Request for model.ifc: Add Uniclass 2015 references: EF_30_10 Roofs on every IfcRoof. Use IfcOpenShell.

First a look at what the model holds.

```python
import ifcopenshell

model = ifcopenshell.open("model.ifc")
print(model.schema)
print("classifications:", [c.Name for c in model.by_type("IfcClassification")])
for ifc_class in ("IfcDoor", "IfcRoof", "IfcStair", "IfcWall", "IfcWindow"):
    print(ifc_class, len(model.by_type(ifc_class)))
```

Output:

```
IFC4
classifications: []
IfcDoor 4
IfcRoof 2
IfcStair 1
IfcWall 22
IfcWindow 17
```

```python
import ifcopenshell
import ifcopenshell.api.classification

model = ifcopenshell.open("model.ifc")

system = ifcopenshell.api.classification.add_classification(model, classification="Uniclass 2015")

codes = {
    "IfcRoof": ("EF_30_10", "Roofs"),
}
for ifc_class, (code, name) in codes.items():
    products = model.by_type(ifc_class)
    ifcopenshell.api.classification.add_reference(
        model, products=products, classification=system, identification=code, name=name
    )
    print(code, len(products))

model.write("model_rev.ifc")
```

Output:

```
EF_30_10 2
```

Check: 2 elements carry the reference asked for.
